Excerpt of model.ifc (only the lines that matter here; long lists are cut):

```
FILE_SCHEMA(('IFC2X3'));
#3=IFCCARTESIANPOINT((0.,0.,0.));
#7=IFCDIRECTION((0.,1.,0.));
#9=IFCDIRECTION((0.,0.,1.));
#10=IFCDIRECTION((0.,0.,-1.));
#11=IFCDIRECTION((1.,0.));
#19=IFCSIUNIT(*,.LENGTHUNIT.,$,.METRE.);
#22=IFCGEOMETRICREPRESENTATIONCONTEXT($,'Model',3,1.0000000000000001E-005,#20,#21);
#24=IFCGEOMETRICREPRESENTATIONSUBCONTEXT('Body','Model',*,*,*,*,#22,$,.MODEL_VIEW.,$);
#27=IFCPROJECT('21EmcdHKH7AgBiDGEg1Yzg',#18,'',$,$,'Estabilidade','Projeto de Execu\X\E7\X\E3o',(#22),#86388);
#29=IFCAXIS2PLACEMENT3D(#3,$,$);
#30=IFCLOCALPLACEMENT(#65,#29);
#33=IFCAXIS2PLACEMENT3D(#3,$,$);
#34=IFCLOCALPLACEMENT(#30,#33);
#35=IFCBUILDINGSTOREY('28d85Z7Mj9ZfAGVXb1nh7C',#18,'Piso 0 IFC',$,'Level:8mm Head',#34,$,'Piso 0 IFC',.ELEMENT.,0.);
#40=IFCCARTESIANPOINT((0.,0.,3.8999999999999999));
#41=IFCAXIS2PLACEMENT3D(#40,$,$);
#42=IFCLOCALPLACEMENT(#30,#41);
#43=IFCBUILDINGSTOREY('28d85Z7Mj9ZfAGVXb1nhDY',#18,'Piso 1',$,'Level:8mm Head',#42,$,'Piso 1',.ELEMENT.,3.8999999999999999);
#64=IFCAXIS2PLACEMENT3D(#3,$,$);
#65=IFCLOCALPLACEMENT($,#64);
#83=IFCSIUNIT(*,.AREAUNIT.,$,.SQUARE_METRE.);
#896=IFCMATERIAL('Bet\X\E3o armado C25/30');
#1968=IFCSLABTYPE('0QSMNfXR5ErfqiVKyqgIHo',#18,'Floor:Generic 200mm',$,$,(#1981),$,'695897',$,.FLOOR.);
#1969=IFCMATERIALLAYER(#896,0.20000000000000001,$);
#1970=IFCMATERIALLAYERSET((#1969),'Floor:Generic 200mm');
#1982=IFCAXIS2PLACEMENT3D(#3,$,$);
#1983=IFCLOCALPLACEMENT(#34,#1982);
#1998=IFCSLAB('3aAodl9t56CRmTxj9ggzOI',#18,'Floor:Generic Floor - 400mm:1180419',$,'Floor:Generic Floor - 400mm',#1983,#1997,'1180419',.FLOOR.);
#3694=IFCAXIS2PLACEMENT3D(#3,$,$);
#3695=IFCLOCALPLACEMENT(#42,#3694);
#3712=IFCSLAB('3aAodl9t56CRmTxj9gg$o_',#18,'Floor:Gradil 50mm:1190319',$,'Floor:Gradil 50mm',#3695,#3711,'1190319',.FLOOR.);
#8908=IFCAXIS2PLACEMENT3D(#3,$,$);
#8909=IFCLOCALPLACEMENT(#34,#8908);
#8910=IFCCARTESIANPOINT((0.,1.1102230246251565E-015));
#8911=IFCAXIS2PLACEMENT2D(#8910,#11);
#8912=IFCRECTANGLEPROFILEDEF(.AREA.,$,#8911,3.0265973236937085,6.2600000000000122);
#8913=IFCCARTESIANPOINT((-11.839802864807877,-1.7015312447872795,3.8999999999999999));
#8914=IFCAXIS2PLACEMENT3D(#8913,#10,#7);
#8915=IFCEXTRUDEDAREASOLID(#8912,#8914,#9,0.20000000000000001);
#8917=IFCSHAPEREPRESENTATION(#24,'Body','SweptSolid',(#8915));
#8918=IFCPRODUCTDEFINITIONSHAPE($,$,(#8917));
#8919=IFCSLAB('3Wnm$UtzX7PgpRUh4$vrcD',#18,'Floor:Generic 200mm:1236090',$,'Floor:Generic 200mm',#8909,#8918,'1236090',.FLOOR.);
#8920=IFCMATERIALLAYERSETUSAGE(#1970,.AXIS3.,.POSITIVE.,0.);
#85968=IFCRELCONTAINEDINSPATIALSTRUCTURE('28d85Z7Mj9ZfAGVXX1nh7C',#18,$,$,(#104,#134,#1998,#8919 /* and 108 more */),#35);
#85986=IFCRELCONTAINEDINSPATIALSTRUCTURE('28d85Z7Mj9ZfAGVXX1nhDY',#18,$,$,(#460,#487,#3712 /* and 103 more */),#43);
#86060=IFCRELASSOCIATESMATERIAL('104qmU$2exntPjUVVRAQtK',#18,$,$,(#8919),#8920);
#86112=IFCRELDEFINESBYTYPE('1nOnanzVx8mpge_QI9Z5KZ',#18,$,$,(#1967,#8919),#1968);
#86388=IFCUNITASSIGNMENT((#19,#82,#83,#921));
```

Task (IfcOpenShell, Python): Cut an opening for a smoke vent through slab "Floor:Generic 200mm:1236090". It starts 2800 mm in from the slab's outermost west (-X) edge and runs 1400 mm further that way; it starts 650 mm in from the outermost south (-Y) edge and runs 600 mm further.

```python
import numpy as np
import ifcopenshell
import ifcopenshell.api.feature
import ifcopenshell.api.geometry
import ifcopenshell.api.root
import ifcopenshell.geom
import ifcopenshell.util.placement
import ifcopenshell.util.representation
import ifcopenshell.util.shape
import ifcopenshell.util.unit

model = ifcopenshell.open("model.ifc")
unit_scale = ifcopenshell.util.unit.calculate_unit_scale(model)
settings = ifcopenshell.geom.settings()


def volume(element):
    """Net volume in cubic metres, openings subtracted."""
    shape = ifcopenshell.geom.create_shape(settings, element)
    return ifcopenshell.util.shape.get_volume(shape.geometry)


slab = model.by_guid("3Wnm$UtzX7PgpRUh4$vrcD")
before = volume(slab)

# Extent in the slab's own axes, in metres. The edges named are its -X and -Y sides.
slab_shape = ifcopenshell.geom.create_shape(settings, slab)
vertices = ifcopenshell.util.shape.get_vertices(slab_shape.geometry)
x_min, y_min, bottom = vertices.min(axis=0)
top = vertices[:, 2].max()

opening = ifcopenshell.api.root.create_entity(model, ifc_class="IfcOpeningElement", name="Smoke vent opening")
context = ifcopenshell.util.representation.get_context(model, "Model", "Body", "MODEL_VIEW")
width, depth = 1.4, 0.6
outline = [(0.0, 0.0), (width, 0.0), (width, depth), (0.0, depth), (0.0, 0.0)]
# Overshoot both faces by 50 mm so the cut is clean.
shape = ifcopenshell.api.geometry.add_slab_representation(
    model, context=context, depth=top - bottom + 0.1, polyline=outline
)
ifcopenshell.api.geometry.assign_representation(model, product=opening, representation=shape)

matrix = ifcopenshell.util.placement.get_local_placement(slab.ObjectPlacement)
matrix[:, 3] = matrix @ np.append(np.array([x_min + 2.8, y_min + 0.65, bottom - 0.05]) / unit_scale, 1.0)
ifcopenshell.api.geometry.edit_object_placement(model, product=opening, matrix=matrix, is_si=False)
ifcopenshell.api.feature.add_feature(model, feature=opening, element=slab)

after = volume(slab)

print(f"slab volume {before:.3f} -> {after:.3f} m3")

model.write("model_updated.ifc")
```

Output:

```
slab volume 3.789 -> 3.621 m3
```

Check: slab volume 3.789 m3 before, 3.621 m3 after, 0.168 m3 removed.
